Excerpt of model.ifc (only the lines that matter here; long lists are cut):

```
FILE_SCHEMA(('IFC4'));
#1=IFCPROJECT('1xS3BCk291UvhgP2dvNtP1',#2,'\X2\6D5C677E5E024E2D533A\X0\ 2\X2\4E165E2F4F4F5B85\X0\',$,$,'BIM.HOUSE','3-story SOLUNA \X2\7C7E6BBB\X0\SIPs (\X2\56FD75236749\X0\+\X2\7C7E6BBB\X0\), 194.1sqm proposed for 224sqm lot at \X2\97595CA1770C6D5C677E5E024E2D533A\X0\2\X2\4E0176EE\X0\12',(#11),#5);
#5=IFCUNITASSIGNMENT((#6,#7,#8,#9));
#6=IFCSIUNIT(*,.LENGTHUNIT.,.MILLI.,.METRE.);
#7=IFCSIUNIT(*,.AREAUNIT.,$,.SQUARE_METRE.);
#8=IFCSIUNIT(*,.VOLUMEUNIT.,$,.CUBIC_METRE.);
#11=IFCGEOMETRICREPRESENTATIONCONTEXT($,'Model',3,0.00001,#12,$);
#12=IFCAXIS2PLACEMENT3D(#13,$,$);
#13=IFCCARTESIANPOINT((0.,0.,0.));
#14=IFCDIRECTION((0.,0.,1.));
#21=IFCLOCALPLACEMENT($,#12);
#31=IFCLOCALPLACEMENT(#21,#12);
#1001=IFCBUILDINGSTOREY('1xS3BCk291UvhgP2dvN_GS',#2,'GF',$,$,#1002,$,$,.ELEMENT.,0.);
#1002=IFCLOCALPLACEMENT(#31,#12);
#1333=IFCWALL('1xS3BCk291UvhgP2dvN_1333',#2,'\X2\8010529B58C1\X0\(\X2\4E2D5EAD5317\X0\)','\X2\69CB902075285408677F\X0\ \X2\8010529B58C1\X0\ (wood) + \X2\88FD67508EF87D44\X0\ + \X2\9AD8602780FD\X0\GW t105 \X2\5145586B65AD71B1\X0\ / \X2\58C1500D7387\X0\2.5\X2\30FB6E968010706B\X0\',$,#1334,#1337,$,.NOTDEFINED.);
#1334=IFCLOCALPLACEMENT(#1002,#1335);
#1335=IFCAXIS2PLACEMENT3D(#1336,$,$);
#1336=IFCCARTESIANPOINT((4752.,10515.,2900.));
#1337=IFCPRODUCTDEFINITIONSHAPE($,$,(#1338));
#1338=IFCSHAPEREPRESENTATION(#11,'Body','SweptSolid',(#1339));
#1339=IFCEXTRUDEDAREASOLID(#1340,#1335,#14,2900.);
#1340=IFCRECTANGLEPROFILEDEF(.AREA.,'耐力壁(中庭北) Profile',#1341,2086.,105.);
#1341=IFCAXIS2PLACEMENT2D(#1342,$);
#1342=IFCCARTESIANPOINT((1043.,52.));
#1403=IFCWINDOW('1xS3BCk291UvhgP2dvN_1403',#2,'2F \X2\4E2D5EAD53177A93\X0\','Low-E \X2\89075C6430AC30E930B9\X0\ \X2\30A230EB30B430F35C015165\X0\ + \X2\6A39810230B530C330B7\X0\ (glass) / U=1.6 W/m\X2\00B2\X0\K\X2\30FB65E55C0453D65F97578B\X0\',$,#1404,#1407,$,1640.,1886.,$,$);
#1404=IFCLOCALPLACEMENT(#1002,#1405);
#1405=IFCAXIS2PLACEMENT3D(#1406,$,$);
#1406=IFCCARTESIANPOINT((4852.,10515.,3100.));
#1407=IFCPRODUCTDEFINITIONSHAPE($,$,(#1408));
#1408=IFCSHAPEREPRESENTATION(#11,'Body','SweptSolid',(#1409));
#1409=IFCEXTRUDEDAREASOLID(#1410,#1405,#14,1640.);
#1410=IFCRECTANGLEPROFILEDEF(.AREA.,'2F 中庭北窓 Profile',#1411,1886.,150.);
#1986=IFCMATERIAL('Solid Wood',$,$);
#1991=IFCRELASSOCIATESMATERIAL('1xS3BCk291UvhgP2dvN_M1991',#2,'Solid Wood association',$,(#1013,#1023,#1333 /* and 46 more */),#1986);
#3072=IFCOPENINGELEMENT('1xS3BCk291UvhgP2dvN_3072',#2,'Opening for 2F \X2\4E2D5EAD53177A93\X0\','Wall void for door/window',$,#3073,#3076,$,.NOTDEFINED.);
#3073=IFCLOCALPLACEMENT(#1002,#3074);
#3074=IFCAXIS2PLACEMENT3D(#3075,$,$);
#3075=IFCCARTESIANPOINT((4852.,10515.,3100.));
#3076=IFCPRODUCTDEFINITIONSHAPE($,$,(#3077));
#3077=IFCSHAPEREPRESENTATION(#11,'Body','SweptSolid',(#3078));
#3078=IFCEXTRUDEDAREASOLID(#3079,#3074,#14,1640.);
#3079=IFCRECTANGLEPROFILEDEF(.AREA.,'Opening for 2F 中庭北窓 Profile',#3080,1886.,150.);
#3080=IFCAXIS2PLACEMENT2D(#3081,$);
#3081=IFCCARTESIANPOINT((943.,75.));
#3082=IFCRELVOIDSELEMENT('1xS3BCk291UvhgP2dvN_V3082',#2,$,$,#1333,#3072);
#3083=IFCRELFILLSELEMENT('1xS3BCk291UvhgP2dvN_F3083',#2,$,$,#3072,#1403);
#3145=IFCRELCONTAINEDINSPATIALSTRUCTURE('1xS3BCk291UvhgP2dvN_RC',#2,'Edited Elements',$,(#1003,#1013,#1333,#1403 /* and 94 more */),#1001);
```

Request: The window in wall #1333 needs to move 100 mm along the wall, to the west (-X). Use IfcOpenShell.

```python
import ifcopenshell
import ifcopenshell.api.geometry
import ifcopenshell.util.placement
import ifcopenshell.util.unit

model = ifcopenshell.open("model.ifc")
unit_scale = ifcopenshell.util.unit.calculate_unit_scale(model)

window = model.by_id(1403)
opening = window.FillsVoids[0].RelatingOpeningElement
wall = opening.VoidsElements[0].RelatingBuildingElement

wall_matrix = ifcopenshell.util.placement.get_local_placement(wall.ObjectPlacement)
shift = wall_matrix[:3, 0] * -0.1 / unit_scale
before = ifcopenshell.util.placement.get_local_placement(window.ObjectPlacement)[:3, 3].copy()

# The window is not placed relative to its opening, so move both.
for product in (opening, window):
    matrix = ifcopenshell.util.placement.get_local_placement(product.ObjectPlacement)
    matrix[:3, 3] += shift
    ifcopenshell.api.geometry.edit_object_placement(model, product=product, matrix=matrix, is_si=False)

after = ifcopenshell.util.placement.get_local_placement(window.ObjectPlacement)[:3, 3]
print("window moved by", (after - before).round(3) + 0.0)

model.write("model_updated.ifc")
```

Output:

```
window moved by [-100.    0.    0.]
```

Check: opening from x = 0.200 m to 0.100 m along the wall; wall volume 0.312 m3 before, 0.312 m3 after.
